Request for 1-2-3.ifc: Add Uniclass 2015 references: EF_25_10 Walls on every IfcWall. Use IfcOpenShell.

First a look at what the model holds.

```python
import ifcopenshell

model = ifcopenshell.open("1-2-3.ifc")
print(model.schema)
print("classifications:", [c.Name for c in model.by_type("IfcClassification")])
for ifc_class in ("IfcDoor", "IfcRoof", "IfcStair", "IfcWall", "IfcWindow"):
    print(ifc_class, len(model.by_type(ifc_class)))
```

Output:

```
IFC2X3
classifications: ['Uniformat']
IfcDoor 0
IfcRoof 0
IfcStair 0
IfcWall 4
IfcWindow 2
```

```python
import ifcopenshell
import ifcopenshell.api.classification

model = ifcopenshell.open("1-2-3.ifc")

# IFC2X3 requires Source and Edition and has no link from the project to the system.
system = model.create_entity("IfcClassification", Source="NBS", Edition="2015", Name="Uniclass 2015")

codes = {
    "IfcWall": ("EF_25_10", "Walls"),
}
for ifc_class, (code, name) in codes.items():
    products = model.by_type(ifc_class)
    ifcopenshell.api.classification.add_reference(
        model, products=products, classification=system, identification=code, name=name
    )
    print(code, len(products))

model.write("1-2-3_edited.ifc")
```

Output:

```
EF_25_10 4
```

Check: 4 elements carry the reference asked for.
